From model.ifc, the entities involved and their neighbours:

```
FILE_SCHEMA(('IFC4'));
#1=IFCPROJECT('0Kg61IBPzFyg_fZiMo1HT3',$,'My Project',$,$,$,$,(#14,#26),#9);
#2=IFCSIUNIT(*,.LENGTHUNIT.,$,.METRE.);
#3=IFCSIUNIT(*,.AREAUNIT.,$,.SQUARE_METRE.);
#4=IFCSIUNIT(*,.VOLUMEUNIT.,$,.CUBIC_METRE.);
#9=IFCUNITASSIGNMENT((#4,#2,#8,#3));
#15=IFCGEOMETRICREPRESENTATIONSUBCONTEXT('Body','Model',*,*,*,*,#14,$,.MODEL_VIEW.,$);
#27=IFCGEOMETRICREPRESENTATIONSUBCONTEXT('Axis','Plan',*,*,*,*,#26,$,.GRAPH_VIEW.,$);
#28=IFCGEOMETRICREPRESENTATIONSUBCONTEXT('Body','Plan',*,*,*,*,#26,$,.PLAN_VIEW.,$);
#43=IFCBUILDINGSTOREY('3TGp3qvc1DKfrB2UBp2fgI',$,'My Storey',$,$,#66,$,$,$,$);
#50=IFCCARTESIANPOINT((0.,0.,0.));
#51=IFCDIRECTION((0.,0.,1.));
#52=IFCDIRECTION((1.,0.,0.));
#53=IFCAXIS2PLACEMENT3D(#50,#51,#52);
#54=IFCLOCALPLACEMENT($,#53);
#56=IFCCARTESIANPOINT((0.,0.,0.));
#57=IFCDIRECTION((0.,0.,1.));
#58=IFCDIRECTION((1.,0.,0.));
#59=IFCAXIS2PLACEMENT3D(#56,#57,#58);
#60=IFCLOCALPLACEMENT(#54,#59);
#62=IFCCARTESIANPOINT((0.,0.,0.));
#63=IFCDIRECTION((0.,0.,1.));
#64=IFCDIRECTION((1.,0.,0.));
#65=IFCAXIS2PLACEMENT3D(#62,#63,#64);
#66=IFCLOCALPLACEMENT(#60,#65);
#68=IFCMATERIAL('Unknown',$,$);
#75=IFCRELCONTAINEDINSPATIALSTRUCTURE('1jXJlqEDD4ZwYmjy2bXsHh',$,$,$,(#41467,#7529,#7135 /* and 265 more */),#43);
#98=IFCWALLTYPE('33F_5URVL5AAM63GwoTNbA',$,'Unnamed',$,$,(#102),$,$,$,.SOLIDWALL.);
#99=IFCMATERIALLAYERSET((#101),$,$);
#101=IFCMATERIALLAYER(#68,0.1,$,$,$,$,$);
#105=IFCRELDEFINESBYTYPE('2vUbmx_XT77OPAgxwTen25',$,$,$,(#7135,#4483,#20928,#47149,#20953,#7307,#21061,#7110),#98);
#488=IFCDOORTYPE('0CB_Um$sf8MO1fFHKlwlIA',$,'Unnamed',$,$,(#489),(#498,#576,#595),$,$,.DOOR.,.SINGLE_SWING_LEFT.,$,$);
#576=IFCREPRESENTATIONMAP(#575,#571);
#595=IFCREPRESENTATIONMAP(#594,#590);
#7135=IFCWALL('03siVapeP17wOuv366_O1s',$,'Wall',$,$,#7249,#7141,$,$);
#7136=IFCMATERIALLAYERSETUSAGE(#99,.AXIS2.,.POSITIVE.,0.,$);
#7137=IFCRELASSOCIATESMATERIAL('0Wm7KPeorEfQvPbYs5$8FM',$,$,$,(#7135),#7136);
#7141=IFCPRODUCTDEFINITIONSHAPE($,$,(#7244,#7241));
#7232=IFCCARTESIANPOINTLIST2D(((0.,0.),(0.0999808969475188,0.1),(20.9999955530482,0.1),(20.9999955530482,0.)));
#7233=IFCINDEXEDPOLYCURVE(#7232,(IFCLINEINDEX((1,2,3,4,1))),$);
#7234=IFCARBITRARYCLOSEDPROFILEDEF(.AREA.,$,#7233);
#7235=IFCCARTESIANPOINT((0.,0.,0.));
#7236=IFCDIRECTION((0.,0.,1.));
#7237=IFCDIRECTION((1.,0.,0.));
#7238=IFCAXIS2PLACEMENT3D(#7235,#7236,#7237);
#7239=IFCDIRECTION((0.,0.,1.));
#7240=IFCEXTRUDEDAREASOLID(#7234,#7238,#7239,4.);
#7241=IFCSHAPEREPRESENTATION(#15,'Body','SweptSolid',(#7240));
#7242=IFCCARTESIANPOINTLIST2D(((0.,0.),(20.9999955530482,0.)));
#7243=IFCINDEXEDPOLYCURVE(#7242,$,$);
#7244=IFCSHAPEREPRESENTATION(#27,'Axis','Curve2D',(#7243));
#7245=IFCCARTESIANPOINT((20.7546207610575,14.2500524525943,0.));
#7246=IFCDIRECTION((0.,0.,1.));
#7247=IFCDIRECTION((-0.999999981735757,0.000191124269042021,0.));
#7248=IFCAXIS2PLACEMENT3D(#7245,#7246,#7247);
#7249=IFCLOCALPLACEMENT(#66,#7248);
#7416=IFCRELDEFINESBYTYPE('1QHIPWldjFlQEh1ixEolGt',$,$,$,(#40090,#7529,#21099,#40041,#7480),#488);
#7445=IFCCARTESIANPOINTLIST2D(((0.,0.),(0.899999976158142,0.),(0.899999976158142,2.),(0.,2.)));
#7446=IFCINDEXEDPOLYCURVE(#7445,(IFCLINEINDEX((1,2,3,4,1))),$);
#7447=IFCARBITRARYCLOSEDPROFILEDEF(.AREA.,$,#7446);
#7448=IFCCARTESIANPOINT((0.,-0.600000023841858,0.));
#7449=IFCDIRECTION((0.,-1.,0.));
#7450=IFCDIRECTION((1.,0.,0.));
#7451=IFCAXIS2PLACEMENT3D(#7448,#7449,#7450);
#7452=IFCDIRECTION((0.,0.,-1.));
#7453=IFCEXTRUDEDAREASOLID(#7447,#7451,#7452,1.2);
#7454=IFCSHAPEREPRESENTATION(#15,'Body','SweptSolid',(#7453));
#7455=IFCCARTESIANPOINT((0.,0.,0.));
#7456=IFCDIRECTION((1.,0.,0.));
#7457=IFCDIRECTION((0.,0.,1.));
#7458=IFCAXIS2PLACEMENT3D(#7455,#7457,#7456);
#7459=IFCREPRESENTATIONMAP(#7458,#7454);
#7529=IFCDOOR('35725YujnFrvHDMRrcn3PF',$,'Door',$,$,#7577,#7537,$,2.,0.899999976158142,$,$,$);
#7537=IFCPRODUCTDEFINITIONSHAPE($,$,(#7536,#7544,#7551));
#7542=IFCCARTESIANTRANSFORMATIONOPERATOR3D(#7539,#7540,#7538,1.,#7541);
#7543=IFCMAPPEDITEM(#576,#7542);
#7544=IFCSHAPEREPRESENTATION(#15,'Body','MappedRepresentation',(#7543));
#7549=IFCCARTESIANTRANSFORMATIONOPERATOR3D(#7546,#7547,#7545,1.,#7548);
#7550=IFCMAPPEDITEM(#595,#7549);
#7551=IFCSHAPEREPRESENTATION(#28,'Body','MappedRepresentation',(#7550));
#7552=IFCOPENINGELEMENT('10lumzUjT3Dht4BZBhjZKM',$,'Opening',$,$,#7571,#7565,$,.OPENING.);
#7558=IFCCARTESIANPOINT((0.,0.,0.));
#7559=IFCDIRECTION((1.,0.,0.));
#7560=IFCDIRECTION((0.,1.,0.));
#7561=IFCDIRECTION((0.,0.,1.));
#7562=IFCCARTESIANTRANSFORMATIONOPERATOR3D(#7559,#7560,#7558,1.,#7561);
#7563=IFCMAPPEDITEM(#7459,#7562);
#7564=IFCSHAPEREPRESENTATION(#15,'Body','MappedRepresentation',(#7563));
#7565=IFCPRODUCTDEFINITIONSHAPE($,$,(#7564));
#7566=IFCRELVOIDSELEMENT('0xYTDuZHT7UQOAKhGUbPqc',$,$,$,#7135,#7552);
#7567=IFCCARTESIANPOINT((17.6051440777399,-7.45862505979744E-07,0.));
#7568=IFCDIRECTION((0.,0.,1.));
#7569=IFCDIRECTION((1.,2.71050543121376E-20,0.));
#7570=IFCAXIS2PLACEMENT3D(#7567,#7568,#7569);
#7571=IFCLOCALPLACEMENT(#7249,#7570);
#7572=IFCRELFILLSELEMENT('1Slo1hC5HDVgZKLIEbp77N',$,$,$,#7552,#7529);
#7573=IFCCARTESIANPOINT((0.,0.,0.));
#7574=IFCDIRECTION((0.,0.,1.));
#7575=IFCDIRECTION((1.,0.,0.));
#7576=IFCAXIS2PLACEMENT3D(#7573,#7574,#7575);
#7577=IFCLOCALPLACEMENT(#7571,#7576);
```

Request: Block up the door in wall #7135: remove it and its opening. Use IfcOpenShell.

```python
import ifcopenshell
import ifcopenshell.api.feature
import ifcopenshell.api.root
import ifcopenshell.geom
import ifcopenshell.util.shape

model = ifcopenshell.open("model.ifc")
settings = ifcopenshell.geom.settings()


def volume(element):
    """Net volume in cubic metres, openings subtracted."""
    shape = ifcopenshell.geom.create_shape(settings, element)
    return ifcopenshell.util.shape.get_volume(shape.geometry)


door = model.by_guid("35725YujnFrvHDMRrcn3PF")
opening = door.FillsVoids[0].RelatingOpeningElement
wall = opening.VoidsElements[0].RelatingBuildingElement
before = volume(wall)

ifcopenshell.api.root.remove_product(model, product=door)
ifcopenshell.api.feature.remove_feature(model, feature=opening)

after = volume(wall)

print(f"wall volume {before:.3f} -> {after:.3f} m3")

model.write("model-out.ifc")
```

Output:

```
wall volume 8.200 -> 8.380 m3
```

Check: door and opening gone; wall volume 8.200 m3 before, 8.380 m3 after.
